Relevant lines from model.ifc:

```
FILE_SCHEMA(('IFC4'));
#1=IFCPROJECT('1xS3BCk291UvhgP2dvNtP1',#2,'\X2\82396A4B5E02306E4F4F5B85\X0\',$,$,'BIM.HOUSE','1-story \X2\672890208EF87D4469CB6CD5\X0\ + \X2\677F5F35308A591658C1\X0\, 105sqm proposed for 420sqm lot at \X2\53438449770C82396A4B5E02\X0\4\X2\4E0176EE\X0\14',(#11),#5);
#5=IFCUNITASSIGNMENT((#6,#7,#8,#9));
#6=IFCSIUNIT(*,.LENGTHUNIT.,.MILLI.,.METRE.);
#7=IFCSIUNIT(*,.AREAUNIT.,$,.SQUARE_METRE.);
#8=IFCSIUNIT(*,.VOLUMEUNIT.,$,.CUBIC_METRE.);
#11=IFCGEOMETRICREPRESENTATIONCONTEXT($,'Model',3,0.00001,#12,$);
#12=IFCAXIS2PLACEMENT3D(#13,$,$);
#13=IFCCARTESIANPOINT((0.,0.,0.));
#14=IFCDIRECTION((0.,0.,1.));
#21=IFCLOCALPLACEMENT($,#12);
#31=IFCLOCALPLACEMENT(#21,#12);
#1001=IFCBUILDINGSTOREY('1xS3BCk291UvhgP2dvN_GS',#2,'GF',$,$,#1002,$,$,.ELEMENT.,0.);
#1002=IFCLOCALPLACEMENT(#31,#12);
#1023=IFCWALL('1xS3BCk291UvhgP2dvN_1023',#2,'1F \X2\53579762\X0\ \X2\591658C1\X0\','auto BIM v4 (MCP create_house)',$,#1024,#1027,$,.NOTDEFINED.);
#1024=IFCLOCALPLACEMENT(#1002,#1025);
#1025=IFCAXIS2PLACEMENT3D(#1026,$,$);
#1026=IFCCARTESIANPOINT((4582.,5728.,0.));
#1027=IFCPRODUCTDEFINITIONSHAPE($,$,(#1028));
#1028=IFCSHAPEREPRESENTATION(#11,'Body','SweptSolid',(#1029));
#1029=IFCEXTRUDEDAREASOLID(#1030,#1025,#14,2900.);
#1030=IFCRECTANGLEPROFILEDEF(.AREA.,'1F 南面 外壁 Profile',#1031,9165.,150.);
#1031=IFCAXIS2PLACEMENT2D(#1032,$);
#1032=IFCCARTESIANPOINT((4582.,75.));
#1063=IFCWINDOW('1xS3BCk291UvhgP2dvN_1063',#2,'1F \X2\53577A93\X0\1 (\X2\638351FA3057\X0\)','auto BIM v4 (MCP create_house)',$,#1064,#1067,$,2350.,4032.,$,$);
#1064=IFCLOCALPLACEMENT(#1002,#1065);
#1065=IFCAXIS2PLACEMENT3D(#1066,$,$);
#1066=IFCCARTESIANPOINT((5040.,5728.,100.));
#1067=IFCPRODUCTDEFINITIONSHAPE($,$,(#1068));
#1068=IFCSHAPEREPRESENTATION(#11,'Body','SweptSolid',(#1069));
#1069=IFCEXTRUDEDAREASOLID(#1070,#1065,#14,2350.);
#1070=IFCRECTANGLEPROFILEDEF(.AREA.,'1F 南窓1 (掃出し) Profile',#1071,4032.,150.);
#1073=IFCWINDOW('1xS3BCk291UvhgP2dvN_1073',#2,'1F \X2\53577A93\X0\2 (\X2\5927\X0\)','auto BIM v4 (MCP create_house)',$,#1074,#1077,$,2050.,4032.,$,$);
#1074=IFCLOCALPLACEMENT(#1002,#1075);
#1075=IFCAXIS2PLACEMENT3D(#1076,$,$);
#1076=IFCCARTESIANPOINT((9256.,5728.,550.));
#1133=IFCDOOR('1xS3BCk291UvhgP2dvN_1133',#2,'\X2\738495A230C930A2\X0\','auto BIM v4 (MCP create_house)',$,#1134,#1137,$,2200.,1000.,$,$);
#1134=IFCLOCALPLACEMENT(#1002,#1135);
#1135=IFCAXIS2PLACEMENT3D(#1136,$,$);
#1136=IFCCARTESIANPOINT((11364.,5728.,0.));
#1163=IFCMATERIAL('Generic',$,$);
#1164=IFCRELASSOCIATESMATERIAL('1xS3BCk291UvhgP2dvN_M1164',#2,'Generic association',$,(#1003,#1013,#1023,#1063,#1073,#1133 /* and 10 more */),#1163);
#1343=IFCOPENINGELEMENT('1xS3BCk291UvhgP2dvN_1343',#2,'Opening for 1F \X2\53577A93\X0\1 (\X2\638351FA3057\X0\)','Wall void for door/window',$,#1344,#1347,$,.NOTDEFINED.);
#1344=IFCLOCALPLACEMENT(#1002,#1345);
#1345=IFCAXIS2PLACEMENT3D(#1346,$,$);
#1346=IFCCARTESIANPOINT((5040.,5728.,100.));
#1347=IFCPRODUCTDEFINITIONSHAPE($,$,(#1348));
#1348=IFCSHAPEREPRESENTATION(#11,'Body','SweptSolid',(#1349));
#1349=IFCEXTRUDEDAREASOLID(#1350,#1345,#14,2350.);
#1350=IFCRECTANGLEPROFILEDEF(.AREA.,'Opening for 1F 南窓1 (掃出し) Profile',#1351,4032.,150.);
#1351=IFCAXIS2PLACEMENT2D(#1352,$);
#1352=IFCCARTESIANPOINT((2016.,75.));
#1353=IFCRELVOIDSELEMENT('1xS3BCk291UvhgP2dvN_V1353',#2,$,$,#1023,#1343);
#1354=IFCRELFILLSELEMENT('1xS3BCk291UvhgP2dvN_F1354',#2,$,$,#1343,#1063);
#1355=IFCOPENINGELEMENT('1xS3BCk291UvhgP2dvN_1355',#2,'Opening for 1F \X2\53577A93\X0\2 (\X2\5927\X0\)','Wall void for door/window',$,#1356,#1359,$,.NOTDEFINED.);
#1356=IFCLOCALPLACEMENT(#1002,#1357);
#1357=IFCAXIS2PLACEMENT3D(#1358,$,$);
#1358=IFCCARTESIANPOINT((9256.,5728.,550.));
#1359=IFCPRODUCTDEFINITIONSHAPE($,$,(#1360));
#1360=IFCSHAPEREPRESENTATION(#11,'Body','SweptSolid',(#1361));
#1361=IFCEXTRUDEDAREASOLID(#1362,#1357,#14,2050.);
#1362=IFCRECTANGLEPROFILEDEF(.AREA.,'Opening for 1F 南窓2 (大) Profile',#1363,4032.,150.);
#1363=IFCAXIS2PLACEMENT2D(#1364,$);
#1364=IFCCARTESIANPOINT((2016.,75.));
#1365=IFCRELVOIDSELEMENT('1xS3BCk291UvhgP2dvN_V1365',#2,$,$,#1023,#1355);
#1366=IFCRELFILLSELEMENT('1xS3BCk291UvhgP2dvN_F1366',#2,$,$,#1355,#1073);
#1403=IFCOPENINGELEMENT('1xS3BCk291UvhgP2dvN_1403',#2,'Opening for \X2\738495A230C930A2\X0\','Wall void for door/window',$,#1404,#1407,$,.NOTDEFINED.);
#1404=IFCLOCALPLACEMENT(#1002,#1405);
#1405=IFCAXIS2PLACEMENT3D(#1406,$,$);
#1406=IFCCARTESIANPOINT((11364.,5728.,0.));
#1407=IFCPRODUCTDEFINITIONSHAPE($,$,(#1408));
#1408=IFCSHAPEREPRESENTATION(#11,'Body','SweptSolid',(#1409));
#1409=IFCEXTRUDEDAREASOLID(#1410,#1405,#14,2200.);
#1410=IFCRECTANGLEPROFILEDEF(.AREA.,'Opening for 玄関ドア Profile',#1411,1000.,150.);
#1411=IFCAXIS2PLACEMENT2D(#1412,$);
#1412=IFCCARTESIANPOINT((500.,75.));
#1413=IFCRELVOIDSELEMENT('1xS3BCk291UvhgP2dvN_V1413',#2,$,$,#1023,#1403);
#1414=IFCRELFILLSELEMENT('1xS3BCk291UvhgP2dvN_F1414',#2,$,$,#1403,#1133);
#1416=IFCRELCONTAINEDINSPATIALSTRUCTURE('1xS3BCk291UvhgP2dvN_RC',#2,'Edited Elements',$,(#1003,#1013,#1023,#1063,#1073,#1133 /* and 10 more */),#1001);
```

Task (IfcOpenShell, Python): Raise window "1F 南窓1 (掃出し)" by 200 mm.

```python
import numpy as np
import ifcopenshell
import ifcopenshell.api.geometry
import ifcopenshell.util.placement
import ifcopenshell.util.unit

model = ifcopenshell.open("model.ifc")
unit_scale = ifcopenshell.util.unit.calculate_unit_scale(model)

window = model.by_id(1063)
opening = window.FillsVoids[0].RelatingOpeningElement
dz = 0.2 / unit_scale

shift = np.array([0.0, 0.0, dz])
# The window is not placed relative to its opening, so move both.
for product in (opening, window):
    matrix = ifcopenshell.util.placement.get_local_placement(product.ObjectPlacement)
    matrix[:3, 3] += shift
    ifcopenshell.api.geometry.edit_object_placement(model, product=product, matrix=matrix, is_si=False)

print(f"moved by {dz * unit_scale:+.3f} m")

model.write("model_edited.ifc")
```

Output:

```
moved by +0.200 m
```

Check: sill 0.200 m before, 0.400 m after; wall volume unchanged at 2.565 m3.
